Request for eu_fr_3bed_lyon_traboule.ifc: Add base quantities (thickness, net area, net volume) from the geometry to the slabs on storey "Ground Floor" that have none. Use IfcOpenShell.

First a look at what the model holds.

```python
import ifcopenshell
import ifcopenshell.util.element
import ifcopenshell.util.unit

model = ifcopenshell.open("eu_fr_3bed_lyon_traboule.ifc")
print(model.schema)
for unit_type in ("LENGTHUNIT", "AREAUNIT", "VOLUMEUNIT"):
    print(unit_type, ifcopenshell.util.unit.calculate_unit_scale(model, unit_type))
storey = next(s for s in model.by_type("IfcBuildingStorey") if s.Name == "Ground Floor")
slabs = [e for e in ifcopenshell.util.element.get_decomposition(storey) if e.is_a("IfcSlab")]
for e in sorted(slabs, key=lambda e: e.id()):
    print(e.id(), e.is_a(), e.Name, list(ifcopenshell.util.element.get_psets(e, qtos_only=True)), sep=" | ")
```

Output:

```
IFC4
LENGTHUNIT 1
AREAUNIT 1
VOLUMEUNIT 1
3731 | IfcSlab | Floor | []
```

```python
import ifcopenshell
import ifcopenshell.api.pset
import ifcopenshell.geom
import ifcopenshell.util.element
import ifcopenshell.util.shape
import ifcopenshell.util.unit

model = ifcopenshell.open("eu_fr_3bed_lyon_traboule.ifc")
unit_scale = ifcopenshell.util.unit.calculate_unit_scale(model)
area_scale = ifcopenshell.util.unit.calculate_unit_scale(model, "AREAUNIT")
volume_scale = ifcopenshell.util.unit.calculate_unit_scale(model, "VOLUMEUNIT")
settings = ifcopenshell.geom.settings()

storey = next(s for s in model.by_type("IfcBuildingStorey") if s.Name == "Ground Floor")
slabs = [e for e in ifcopenshell.util.element.get_decomposition(storey) if e.is_a("IfcSlab")]

for e in sorted(slabs, key=lambda e: e.id()):
    if ifcopenshell.util.element.get_psets(e, qtos_only=True, should_inherit=False):
        continue
    # Geometry comes back in metres, in the element's own axes.
    shape = ifcopenshell.geom.create_shape(settings, e)
    values = {
        "Width": ifcopenshell.util.shape.get_z(shape.geometry) / unit_scale,
        "NetArea": ifcopenshell.util.shape.get_footprint_area(shape.geometry) / area_scale,
        "NetVolume": ifcopenshell.util.shape.get_volume(shape.geometry) / volume_scale,
    }
    qto = ifcopenshell.api.pset.add_qto(model, product=e, name="Qto_SlabBaseQuantities")
    ifcopenshell.api.pset.edit_qto(model, qto=qto, properties=values)
    print(e.id(), {k: round(v, 3) for k, v in values.items()})

model.write("eu_fr_3bed_lyon_traboule_edited.ifc")
```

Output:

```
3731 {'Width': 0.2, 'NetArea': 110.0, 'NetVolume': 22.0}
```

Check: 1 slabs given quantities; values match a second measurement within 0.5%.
